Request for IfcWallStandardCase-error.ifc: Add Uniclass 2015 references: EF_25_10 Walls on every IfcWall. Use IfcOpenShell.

First a look at what the model holds.

```python
import ifcopenshell

model = ifcopenshell.open("IfcWallStandardCase-error.ifc")
print(model.schema)
print("classifications:", [c.Name for c in model.by_type("IfcClassification")])
for ifc_class in ("IfcDoor", "IfcRoof", "IfcStair", "IfcWall", "IfcWindow"):
    print(ifc_class, len(model.by_type(ifc_class)))
```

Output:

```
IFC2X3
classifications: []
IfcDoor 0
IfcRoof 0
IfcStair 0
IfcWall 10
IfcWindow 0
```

```python
import ifcopenshell
import ifcopenshell.api.classification

model = ifcopenshell.open("IfcWallStandardCase-error.ifc")

# IFC2X3 requires Source and Edition and has no link from the project to the system.
system = model.create_entity("IfcClassification", Source="NBS", Edition="2015", Name="Uniclass 2015")

codes = {
    "IfcWall": ("EF_25_10", "Walls"),
}
for ifc_class, (code, name) in codes.items():
    products = model.by_type(ifc_class)
    ifcopenshell.api.classification.add_reference(
        model, products=products, classification=system, identification=code, name=name
    )
    print(code, len(products))

model.write("IfcWallStandardCase-error-out.ifc")
```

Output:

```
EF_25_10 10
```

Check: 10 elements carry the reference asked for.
